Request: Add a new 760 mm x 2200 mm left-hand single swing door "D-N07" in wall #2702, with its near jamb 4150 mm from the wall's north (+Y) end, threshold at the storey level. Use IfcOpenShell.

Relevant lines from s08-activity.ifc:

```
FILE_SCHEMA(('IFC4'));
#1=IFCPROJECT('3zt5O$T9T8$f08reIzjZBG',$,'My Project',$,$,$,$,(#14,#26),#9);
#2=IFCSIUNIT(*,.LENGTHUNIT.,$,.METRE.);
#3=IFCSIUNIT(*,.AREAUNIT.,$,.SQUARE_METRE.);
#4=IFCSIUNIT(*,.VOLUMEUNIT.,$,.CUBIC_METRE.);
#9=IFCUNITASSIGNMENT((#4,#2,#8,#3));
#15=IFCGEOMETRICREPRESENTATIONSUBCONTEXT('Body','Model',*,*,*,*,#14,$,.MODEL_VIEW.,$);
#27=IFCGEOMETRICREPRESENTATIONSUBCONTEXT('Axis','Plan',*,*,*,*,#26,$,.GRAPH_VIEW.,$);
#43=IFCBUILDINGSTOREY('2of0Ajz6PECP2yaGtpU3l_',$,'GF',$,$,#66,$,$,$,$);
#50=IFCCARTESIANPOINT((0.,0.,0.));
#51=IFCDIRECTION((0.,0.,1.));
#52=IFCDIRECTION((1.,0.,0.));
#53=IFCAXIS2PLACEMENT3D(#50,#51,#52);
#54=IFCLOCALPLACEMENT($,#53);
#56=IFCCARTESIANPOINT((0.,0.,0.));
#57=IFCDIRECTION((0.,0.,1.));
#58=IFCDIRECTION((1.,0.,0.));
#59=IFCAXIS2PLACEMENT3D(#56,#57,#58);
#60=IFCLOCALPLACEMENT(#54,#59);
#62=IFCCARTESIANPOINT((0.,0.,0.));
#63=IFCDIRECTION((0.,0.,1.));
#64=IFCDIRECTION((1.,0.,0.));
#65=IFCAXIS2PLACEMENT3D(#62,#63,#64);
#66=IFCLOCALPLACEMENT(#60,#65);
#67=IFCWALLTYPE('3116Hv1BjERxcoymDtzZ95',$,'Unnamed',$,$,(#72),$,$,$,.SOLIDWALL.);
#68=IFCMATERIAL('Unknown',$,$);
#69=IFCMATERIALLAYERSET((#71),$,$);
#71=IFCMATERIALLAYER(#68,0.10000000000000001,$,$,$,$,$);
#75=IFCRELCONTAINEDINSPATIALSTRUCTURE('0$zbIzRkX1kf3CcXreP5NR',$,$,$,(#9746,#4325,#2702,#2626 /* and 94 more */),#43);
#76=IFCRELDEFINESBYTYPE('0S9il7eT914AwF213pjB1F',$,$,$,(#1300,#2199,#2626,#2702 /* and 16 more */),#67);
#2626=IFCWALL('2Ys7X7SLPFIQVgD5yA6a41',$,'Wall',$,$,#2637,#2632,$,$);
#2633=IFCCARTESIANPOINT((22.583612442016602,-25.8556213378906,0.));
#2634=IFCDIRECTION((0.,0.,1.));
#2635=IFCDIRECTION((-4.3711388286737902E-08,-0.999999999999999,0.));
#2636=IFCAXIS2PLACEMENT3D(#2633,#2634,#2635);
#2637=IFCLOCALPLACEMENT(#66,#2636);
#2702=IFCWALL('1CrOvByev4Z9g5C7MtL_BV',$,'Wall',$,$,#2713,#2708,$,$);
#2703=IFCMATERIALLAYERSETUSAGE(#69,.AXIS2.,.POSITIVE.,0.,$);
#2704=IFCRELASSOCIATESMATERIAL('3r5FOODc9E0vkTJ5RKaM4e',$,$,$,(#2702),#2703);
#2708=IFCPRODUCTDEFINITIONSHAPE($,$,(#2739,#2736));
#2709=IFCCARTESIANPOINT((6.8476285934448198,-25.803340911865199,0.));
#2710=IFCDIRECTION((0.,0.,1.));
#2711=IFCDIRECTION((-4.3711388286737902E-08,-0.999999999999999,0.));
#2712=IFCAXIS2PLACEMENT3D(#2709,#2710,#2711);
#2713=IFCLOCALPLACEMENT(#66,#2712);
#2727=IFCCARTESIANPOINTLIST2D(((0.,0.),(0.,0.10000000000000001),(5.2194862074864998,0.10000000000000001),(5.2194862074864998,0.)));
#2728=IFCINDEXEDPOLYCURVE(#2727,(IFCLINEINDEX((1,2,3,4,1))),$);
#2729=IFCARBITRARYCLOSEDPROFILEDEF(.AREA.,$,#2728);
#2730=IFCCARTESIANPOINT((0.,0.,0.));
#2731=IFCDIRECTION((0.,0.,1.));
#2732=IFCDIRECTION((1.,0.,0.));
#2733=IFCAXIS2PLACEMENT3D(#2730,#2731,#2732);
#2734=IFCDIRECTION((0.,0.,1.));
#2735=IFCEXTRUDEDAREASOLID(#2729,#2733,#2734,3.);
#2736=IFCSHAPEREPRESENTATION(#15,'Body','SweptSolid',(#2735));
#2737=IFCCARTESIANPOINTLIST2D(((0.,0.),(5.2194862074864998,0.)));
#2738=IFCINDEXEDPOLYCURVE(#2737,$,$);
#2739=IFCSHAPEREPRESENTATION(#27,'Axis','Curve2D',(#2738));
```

```python
import numpy as np
import ifcopenshell
import ifcopenshell.api.feature
import ifcopenshell.api.geometry
import ifcopenshell.api.root
import ifcopenshell.api.spatial
import ifcopenshell.geom
import ifcopenshell.util.element
import ifcopenshell.util.placement
import ifcopenshell.util.representation
import ifcopenshell.util.shape
import ifcopenshell.util.unit

model = ifcopenshell.open("s08-activity.ifc")
unit_scale = ifcopenshell.util.unit.calculate_unit_scale(model)
settings = ifcopenshell.geom.settings()


def volume(element):
    """Net volume in cubic metres, openings subtracted."""
    shape = ifcopenshell.geom.create_shape(settings, element)
    return ifcopenshell.util.shape.get_volume(shape.geometry)


wall = model.by_guid("1CrOvByev4Z9g5C7MtL_BV")
storey = ifcopenshell.util.element.get_container(wall, ifc_class="IfcBuildingStorey")
context = ifcopenshell.util.representation.get_context(model, "Model", "Body", "MODEL_VIEW")
before = volume(wall)

width, height, from_end, sill = 0.76, 2.2, 4.15, 0.0  # metres

# The wall runs along its own X axis, and the end named is its -X end.
wall_shape = ifcopenshell.geom.create_shape(settings, wall)
x, y, z = ifcopenshell.util.shape.get_vertices(wall_shape.geometry).T
start = x.min() + from_end
face, thickness = float(y.min()), float(y.max() - y.min())
wall_matrix = ifcopenshell.util.placement.get_local_placement(wall.ObjectPlacement)
level = ifcopenshell.util.placement.get_local_placement(storey.ObjectPlacement)[2, 3]


def in_wall(x, y):
    """Placement at x, y metres in the wall's axes, at sill height."""
    matrix = wall_matrix.copy()
    matrix[:, 3] = wall_matrix @ np.array([x / unit_scale, y / unit_scale, 0.0, 1.0])
    matrix[2, 3] = level + sill / unit_scale
    return matrix


# Opening: a box that overshoots both wall faces by 50 mm.
opening = ifcopenshell.api.root.create_entity(model, ifc_class="IfcOpeningElement", predefined_type="OPENING")
box = ifcopenshell.api.geometry.add_wall_representation(
    model, context=context, length=width, height=height, thickness=thickness + 0.1
)
ifcopenshell.api.geometry.assign_representation(model, product=opening, representation=box)
ifcopenshell.api.geometry.edit_object_placement(model, product=opening, matrix=in_wall(start, face - 0.05), is_si=False)
ifcopenshell.api.feature.add_feature(model, feature=opening, element=wall)

door = ifcopenshell.api.root.create_entity(model, ifc_class="IfcDoor", name="D-N07", predefined_type="DOOR")
door.OverallWidth, door.OverallHeight = width / unit_scale, height / unit_scale
door.OperationType = "SINGLE_SWING_LEFT"
body = ifcopenshell.api.geometry.add_door_representation(
    model,
    context=context,
    overall_width=door.OverallWidth,
    overall_height=door.OverallHeight,
    operation_type="SINGLE_SWING_LEFT",
    lining_properties={"LiningDepth": thickness / unit_scale, "ThresholdDepth": thickness / unit_scale},
)
ifcopenshell.api.geometry.assign_representation(model, product=door, representation=body)
ifcopenshell.api.spatial.assign_container(model, products=[door], relating_structure=storey)
ifcopenshell.api.feature.add_filling(model, opening=opening, element=door)

# The lining spans the wall, so the door starts at the wall face.
ifcopenshell.api.geometry.edit_object_placement(model, product=door, matrix=in_wall(start, face), is_si=False)

after = volume(wall)

print(f"wall volume {before:.3f} -> {after:.3f} m3")

model.write("s08-activity-out.ifc")
```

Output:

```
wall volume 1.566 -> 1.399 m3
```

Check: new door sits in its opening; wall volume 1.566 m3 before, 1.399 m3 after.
